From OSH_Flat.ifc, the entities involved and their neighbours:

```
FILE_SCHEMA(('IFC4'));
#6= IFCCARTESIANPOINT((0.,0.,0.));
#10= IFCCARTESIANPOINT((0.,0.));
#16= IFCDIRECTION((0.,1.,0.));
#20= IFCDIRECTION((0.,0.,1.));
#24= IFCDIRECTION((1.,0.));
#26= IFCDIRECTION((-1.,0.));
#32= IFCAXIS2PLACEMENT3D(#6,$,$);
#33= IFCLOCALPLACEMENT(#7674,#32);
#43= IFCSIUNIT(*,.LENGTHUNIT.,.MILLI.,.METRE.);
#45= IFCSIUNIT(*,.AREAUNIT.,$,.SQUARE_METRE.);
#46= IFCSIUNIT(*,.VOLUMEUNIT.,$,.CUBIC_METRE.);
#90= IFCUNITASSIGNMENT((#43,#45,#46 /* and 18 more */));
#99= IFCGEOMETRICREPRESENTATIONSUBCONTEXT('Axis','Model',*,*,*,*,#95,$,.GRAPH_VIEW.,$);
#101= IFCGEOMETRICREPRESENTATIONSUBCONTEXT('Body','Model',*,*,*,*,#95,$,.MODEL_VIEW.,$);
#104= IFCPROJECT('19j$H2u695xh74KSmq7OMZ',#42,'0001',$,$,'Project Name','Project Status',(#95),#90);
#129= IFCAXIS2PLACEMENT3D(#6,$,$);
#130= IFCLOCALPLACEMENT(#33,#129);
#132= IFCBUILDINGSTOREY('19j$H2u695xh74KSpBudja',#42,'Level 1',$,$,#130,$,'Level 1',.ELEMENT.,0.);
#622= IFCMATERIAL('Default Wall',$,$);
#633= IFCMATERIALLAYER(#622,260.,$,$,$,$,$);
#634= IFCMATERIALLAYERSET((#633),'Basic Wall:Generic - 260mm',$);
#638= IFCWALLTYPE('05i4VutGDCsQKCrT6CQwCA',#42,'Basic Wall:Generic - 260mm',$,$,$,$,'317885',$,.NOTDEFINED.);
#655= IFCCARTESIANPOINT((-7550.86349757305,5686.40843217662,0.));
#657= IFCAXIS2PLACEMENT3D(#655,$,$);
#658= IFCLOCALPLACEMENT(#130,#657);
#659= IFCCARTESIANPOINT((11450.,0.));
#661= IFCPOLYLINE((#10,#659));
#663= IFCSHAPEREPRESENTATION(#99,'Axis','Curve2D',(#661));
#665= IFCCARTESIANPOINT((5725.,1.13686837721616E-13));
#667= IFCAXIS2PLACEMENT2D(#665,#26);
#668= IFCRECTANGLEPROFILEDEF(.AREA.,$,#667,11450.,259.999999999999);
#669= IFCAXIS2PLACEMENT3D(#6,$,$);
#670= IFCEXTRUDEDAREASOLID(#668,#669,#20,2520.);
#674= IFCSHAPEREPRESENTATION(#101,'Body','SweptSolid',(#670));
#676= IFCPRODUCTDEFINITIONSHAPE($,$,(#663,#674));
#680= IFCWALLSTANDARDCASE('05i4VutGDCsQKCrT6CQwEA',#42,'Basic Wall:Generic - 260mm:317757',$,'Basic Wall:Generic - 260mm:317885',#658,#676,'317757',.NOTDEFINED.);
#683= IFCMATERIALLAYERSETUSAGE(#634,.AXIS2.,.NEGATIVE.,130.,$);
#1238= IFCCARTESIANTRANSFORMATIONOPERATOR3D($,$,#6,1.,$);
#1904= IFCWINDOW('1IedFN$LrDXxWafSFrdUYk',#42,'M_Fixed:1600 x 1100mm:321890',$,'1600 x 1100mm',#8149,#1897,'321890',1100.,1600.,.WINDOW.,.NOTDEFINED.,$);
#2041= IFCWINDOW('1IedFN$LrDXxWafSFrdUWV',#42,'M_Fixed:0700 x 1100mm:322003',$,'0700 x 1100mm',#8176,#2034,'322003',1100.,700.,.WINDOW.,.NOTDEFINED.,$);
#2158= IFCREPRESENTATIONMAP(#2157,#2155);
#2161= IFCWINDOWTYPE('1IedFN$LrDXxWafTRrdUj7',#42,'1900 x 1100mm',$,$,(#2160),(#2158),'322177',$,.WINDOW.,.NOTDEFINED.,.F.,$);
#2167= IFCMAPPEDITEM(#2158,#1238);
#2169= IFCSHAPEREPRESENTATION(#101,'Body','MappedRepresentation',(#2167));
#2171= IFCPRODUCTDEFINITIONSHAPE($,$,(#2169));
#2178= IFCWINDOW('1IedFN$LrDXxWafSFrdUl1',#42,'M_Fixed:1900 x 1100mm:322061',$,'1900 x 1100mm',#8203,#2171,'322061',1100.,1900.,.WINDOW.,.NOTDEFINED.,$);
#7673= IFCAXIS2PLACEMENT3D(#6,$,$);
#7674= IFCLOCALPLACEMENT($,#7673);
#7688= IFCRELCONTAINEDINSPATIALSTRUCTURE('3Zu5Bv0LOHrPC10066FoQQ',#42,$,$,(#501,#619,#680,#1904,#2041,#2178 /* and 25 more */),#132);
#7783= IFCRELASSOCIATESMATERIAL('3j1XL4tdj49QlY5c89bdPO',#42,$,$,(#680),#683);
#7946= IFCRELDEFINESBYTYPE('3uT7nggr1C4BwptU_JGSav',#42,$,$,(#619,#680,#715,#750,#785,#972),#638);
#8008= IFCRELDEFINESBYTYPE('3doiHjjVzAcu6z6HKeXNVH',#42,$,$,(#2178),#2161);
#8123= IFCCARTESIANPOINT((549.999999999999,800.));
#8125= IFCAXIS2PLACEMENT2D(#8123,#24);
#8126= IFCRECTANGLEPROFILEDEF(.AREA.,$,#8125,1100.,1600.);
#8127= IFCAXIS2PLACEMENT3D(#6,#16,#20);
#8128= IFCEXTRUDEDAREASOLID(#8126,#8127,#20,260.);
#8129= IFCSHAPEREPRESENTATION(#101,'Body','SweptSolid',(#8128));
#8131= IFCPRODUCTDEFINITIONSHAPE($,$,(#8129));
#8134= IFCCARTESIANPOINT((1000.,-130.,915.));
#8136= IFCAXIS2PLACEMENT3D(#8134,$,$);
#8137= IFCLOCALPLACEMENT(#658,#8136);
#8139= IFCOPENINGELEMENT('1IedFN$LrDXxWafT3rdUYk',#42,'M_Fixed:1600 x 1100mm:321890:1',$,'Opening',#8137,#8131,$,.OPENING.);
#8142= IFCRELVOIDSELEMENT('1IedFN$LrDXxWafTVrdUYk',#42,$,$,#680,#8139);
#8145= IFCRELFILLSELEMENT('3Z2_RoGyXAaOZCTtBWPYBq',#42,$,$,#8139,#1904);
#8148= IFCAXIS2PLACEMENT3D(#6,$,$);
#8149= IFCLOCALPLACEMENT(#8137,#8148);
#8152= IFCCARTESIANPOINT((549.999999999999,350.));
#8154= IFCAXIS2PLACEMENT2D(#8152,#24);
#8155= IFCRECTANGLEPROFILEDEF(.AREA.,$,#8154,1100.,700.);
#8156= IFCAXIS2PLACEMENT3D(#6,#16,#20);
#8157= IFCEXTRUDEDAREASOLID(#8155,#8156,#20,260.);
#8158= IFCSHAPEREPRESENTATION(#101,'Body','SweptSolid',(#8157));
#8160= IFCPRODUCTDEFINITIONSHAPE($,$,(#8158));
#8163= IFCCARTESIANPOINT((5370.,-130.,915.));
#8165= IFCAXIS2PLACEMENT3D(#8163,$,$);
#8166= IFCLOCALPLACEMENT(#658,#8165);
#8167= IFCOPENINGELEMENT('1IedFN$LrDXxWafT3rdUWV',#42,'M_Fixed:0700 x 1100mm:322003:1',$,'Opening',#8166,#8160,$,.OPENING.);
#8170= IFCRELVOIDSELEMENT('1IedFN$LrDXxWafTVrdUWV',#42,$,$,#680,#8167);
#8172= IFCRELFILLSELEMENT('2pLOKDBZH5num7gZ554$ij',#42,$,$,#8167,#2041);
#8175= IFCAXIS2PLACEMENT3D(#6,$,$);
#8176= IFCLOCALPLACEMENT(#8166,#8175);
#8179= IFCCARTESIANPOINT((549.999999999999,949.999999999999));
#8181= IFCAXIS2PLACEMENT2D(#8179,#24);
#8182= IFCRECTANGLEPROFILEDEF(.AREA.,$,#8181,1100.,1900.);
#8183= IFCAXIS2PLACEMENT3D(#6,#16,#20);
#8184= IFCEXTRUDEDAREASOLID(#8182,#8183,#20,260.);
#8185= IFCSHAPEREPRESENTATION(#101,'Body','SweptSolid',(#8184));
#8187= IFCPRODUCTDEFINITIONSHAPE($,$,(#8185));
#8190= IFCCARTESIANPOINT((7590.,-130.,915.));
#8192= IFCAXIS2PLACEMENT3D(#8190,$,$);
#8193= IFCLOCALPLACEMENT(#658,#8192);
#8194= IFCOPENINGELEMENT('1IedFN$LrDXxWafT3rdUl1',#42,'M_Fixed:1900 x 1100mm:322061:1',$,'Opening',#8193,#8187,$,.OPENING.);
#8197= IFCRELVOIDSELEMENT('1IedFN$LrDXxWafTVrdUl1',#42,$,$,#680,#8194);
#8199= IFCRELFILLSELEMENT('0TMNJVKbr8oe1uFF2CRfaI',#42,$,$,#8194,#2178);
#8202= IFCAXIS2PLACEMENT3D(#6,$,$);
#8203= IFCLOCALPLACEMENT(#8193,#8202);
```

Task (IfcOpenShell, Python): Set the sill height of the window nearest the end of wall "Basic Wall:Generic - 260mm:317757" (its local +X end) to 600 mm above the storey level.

```python
import numpy as np
import ifcopenshell
import ifcopenshell.api.geometry
import ifcopenshell.geom
import ifcopenshell.util.element
import ifcopenshell.util.placement
import ifcopenshell.util.shape
import ifcopenshell.util.unit

model = ifcopenshell.open("OSH_Flat.ifc")
unit_scale = ifcopenshell.util.unit.calculate_unit_scale(model)

window = model.by_id(2178)
opening = window.FillsVoids[0].RelatingOpeningElement
storey = ifcopenshell.util.element.get_container(window, ifc_class="IfcBuildingStorey")
level = ifcopenshell.util.placement.get_local_placement(storey.ObjectPlacement)[2, 3]

# The opening's origin need not be at the sill, so measure its lowest point.
shape = ifcopenshell.geom.create_shape(ifcopenshell.geom.settings(), opening)
bottom = ifcopenshell.util.shape.get_shape_bottom_elevation(shape, shape.geometry) / unit_scale
dz = level + 0.6 / unit_scale - bottom

shift = np.array([0.0, 0.0, dz])
# The window is placed relative to its opening, so it follows when the opening moves.
matrix = ifcopenshell.util.placement.get_local_placement(opening.ObjectPlacement)
matrix[:3, 3] += shift
ifcopenshell.api.geometry.edit_object_placement(
    model, product=opening, matrix=matrix, is_si=False, should_transform_children=True
)

print(f"moved by {dz * unit_scale:+.3f} m")

model.write("OSH_Flat-out.ifc")
```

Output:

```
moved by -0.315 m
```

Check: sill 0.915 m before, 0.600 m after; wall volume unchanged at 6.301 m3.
